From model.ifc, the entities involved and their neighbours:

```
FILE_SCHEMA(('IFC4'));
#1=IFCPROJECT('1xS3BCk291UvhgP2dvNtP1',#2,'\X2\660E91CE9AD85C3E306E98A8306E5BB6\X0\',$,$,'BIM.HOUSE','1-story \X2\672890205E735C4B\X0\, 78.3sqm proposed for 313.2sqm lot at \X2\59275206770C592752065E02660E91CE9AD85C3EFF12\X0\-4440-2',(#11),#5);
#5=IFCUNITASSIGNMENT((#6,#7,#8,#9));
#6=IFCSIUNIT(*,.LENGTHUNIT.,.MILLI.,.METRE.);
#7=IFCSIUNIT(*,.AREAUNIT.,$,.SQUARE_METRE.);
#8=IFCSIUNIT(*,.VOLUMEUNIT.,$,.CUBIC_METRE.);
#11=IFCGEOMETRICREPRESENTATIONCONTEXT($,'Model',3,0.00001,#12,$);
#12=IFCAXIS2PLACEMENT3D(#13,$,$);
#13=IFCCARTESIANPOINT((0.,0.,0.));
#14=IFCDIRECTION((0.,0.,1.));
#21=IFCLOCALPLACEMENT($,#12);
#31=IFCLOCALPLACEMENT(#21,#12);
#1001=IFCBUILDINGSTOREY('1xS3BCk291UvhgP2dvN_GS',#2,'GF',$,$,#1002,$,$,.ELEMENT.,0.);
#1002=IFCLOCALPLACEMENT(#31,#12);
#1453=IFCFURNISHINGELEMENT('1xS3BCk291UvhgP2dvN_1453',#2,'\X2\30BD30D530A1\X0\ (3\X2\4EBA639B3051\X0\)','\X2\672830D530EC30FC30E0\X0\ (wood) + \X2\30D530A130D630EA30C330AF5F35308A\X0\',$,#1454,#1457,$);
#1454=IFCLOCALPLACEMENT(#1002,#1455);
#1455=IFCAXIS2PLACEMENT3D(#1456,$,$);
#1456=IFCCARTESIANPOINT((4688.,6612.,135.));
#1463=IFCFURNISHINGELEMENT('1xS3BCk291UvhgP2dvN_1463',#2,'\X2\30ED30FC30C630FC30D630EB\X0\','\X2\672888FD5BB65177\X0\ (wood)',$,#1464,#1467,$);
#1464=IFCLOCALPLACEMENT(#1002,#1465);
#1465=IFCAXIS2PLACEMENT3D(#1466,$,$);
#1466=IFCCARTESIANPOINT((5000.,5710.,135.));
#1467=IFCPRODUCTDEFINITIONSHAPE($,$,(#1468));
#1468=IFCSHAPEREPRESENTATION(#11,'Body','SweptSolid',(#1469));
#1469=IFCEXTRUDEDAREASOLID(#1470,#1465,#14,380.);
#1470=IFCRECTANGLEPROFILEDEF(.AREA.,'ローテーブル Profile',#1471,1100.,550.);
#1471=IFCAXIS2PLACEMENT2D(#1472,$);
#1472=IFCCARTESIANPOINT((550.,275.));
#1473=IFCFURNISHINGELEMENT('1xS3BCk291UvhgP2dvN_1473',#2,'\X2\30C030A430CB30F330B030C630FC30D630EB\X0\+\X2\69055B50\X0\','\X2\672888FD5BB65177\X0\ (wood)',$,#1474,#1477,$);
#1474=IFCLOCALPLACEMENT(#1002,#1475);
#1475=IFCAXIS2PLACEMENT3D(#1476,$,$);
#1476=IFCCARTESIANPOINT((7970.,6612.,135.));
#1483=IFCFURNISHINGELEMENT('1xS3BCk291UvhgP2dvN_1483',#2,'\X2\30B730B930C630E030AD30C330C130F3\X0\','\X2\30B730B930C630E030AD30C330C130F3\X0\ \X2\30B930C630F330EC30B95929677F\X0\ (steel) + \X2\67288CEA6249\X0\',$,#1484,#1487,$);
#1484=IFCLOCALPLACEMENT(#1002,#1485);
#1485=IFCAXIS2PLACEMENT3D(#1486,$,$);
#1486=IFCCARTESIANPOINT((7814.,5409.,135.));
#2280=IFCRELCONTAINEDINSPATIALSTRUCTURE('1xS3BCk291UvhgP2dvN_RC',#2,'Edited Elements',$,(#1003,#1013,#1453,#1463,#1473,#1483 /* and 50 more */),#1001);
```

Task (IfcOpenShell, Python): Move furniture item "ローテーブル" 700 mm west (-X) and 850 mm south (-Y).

```python
import ifcopenshell
import ifcopenshell.api.geometry
import ifcopenshell.util.placement

model = ifcopenshell.open("model.ifc")

item = model.by_id(1463)
matrix = ifcopenshell.util.placement.get_local_placement(item.ObjectPlacement)
matrix[0, 3] -= 700.0
matrix[1, 3] -= 850.0
ifcopenshell.api.geometry.edit_object_placement(model, product=item, matrix=matrix, is_si=False)

print(ifcopenshell.util.placement.get_local_placement(item.ObjectPlacement).round(3) + 0.0)

model.write("model-out.ifc")
```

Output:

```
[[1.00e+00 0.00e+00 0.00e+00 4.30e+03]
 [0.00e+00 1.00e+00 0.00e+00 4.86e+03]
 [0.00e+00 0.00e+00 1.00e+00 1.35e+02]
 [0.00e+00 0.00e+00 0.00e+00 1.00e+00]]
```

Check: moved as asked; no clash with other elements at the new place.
